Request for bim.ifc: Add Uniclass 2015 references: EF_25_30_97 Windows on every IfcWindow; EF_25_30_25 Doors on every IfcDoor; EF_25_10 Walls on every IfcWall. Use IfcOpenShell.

First a look at what the model holds.

```python
import ifcopenshell

model = ifcopenshell.open("bim.ifc")
print(model.schema)
print("classifications:", [c.Name for c in model.by_type("IfcClassification")])
for ifc_class in ("IfcDoor", "IfcRoof", "IfcStair", "IfcWall", "IfcWindow"):
    print(ifc_class, len(model.by_type(ifc_class)))
```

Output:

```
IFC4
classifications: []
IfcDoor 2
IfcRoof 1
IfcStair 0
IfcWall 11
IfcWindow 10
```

```python
import ifcopenshell
import ifcopenshell.api.classification

model = ifcopenshell.open("bim.ifc")

system = ifcopenshell.api.classification.add_classification(model, classification="Uniclass 2015")

codes = {
    "IfcWindow": ("EF_25_30_97", "Windows"),
    "IfcDoor": ("EF_25_30_25", "Doors"),
    "IfcWall": ("EF_25_10", "Walls"),
}
for ifc_class, (code, name) in codes.items():
    products = model.by_type(ifc_class)
    ifcopenshell.api.classification.add_reference(
        model, products=products, classification=system, identification=code, name=name
    )
    print(code, len(products))

model.write("bim-out.ifc")
```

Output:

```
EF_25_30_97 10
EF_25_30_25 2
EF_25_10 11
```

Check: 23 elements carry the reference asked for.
